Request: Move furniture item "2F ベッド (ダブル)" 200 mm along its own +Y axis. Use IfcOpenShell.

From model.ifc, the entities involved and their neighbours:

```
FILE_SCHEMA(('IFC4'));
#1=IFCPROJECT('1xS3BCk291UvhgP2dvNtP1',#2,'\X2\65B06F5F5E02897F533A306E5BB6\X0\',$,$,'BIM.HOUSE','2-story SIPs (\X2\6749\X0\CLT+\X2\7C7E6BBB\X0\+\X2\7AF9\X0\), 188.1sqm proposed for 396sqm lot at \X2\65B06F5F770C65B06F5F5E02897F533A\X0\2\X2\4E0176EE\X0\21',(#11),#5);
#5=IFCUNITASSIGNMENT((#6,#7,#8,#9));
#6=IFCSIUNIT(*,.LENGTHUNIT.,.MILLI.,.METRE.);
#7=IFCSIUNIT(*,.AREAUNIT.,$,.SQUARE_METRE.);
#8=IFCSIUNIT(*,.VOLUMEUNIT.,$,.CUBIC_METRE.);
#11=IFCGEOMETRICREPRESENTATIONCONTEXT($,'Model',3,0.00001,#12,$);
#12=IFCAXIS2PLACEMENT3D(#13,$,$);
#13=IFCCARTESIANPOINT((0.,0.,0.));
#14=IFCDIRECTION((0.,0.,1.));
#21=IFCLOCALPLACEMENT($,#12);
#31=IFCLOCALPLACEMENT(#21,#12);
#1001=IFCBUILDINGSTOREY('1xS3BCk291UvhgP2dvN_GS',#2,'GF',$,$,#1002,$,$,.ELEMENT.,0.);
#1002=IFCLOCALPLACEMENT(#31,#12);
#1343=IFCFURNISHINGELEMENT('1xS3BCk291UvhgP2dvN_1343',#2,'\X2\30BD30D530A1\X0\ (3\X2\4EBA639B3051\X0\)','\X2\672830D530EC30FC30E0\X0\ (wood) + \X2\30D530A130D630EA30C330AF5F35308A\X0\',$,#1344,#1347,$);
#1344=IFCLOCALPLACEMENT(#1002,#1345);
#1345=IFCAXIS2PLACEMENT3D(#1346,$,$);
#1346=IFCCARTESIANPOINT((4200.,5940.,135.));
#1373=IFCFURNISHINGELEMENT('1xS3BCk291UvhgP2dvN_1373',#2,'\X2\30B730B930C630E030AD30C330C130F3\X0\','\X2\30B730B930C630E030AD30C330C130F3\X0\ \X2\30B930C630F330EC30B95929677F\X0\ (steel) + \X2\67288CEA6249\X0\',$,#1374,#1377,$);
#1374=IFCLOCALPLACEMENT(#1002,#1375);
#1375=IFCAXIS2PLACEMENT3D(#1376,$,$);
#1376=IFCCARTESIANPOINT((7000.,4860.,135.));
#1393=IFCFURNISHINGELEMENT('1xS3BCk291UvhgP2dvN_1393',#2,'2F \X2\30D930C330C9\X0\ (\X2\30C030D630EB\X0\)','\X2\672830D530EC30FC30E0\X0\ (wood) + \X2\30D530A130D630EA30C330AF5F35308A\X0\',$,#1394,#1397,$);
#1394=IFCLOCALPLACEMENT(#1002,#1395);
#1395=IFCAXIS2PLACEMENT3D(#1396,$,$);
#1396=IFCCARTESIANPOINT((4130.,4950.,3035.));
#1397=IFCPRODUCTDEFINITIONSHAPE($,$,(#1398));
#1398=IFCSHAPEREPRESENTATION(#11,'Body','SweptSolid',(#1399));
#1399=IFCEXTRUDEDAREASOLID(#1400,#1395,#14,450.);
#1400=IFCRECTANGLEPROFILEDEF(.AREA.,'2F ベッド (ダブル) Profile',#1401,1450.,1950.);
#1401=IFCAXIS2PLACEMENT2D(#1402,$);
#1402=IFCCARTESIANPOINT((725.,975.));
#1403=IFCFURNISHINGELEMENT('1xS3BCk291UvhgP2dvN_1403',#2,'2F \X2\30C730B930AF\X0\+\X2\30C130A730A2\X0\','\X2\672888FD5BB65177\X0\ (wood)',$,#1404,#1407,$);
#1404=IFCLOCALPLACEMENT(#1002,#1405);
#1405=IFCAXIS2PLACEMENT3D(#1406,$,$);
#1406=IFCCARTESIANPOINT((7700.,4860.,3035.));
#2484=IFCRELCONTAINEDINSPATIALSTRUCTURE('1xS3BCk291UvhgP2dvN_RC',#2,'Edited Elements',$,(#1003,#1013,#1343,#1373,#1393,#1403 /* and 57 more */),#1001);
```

```python
import ifcopenshell
import ifcopenshell.api.geometry
import ifcopenshell.util.placement
import ifcopenshell.util.unit

model = ifcopenshell.open("model.ifc")
unit_scale = ifcopenshell.util.unit.calculate_unit_scale(model)

item = model.by_guid("1xS3BCk291UvhgP2dvN_1393")
matrix = ifcopenshell.util.placement.get_local_placement(item.ObjectPlacement)
matrix[:3, 3] += matrix[:3, 1] * 0.2 / unit_scale
ifcopenshell.api.geometry.edit_object_placement(model, product=item, matrix=matrix, is_si=False)

print(ifcopenshell.util.placement.get_local_placement(item.ObjectPlacement).round(3) + 0.0)

model.write("model_rev.ifc")
```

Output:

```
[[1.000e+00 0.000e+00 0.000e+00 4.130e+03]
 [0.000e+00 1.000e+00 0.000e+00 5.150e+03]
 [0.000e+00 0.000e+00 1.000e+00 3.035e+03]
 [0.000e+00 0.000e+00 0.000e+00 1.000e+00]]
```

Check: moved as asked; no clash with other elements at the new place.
